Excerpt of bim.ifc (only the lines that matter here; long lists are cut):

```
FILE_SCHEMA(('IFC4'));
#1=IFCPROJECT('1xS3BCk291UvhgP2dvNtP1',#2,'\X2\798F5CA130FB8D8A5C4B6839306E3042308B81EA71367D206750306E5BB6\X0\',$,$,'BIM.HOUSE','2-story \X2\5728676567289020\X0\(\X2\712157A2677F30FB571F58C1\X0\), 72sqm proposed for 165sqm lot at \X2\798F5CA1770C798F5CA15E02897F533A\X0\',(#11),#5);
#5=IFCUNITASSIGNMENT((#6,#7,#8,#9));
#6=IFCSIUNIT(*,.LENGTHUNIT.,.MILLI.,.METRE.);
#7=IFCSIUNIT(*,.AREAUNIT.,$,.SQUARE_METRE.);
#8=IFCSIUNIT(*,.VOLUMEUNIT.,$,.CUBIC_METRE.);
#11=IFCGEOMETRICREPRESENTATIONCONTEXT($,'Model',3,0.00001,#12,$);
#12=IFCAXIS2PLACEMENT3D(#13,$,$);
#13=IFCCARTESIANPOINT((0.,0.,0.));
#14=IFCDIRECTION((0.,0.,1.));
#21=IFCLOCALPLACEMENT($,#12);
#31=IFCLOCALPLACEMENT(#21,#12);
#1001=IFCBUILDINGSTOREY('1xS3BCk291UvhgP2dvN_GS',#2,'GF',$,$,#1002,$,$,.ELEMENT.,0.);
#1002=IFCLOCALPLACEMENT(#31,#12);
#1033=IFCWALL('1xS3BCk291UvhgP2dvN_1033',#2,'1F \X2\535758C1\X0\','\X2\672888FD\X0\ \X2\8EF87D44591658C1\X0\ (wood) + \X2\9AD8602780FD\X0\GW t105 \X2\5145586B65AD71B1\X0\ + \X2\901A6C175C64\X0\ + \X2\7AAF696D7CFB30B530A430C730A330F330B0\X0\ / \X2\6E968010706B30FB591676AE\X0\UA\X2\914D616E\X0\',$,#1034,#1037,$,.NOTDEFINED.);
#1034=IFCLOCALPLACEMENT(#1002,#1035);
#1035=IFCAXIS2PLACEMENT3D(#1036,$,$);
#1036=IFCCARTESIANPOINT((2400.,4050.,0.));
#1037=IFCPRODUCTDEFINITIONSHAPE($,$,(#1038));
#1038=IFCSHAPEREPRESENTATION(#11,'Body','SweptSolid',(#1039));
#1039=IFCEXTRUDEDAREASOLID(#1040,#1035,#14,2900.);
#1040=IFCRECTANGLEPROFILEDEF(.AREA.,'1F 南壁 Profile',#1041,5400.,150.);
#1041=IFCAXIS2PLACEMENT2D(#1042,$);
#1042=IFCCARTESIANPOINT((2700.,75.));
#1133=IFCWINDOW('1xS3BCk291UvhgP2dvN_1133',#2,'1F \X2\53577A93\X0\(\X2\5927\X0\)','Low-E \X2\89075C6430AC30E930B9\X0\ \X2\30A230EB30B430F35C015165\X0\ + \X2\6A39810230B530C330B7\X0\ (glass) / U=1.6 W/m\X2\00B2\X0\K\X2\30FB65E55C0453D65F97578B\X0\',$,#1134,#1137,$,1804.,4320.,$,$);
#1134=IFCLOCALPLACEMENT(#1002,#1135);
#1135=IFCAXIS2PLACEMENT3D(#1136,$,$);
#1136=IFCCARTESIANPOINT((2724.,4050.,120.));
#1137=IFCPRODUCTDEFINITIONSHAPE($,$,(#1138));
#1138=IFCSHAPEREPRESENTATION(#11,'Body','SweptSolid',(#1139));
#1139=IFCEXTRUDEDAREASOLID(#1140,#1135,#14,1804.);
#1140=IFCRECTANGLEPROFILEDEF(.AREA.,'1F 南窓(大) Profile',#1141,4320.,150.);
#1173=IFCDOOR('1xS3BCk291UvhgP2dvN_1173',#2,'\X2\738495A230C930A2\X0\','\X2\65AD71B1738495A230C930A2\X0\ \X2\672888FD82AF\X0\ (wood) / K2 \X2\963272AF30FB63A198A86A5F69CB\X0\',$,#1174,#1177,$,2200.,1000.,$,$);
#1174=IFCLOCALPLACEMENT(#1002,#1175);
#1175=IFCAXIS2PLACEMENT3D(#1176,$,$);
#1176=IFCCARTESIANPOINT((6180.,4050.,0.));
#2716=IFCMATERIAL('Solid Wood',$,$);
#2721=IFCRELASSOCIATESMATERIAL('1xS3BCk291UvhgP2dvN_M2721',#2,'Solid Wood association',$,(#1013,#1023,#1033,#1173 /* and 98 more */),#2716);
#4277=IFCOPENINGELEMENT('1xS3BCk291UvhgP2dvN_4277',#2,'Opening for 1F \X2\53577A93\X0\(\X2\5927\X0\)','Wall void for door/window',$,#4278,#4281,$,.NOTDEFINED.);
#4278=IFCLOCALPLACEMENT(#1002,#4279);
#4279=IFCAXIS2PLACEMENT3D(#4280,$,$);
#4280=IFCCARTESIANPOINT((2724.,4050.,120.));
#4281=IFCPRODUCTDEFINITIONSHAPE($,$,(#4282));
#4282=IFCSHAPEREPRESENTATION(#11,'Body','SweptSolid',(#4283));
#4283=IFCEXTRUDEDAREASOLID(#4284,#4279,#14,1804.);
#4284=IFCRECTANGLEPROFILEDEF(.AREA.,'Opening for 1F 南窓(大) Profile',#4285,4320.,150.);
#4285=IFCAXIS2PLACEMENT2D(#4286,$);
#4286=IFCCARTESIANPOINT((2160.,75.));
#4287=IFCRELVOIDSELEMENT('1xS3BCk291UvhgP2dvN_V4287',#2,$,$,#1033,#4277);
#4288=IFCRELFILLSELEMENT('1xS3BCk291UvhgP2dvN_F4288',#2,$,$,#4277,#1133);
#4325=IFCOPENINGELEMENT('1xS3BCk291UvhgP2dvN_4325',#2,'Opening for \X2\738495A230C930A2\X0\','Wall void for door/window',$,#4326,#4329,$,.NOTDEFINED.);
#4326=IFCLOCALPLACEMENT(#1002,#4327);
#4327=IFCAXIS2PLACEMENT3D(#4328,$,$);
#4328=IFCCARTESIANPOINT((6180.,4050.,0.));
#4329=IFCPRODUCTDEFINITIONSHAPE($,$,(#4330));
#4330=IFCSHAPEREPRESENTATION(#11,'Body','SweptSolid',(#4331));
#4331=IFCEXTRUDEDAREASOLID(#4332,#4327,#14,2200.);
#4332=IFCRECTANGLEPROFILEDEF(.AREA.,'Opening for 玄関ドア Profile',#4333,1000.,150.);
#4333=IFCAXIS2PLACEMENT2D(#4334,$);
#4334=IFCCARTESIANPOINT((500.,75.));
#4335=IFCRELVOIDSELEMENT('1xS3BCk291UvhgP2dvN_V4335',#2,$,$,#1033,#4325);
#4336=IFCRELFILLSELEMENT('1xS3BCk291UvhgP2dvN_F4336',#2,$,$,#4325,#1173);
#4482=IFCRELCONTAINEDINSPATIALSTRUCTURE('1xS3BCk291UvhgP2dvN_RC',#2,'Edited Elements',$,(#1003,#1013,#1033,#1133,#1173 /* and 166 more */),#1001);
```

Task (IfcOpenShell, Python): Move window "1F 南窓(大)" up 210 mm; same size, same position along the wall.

```python
import numpy as np
import ifcopenshell
import ifcopenshell.api.geometry
import ifcopenshell.util.placement
import ifcopenshell.util.unit

model = ifcopenshell.open("bim.ifc")
unit_scale = ifcopenshell.util.unit.calculate_unit_scale(model)

window = model.by_guid("1xS3BCk291UvhgP2dvN_1133")
opening = window.FillsVoids[0].RelatingOpeningElement
dz = 0.21 / unit_scale

shift = np.array([0.0, 0.0, dz])
# The window is not placed relative to its opening, so move both.
for product in (opening, window):
    matrix = ifcopenshell.util.placement.get_local_placement(product.ObjectPlacement)
    matrix[:3, 3] += shift
    ifcopenshell.api.geometry.edit_object_placement(model, product=product, matrix=matrix, is_si=False)

print(f"moved by {dz * unit_scale:+.3f} m")

model.write("bim_edited.ifc")
```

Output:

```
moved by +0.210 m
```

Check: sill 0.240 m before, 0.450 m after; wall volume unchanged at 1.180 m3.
